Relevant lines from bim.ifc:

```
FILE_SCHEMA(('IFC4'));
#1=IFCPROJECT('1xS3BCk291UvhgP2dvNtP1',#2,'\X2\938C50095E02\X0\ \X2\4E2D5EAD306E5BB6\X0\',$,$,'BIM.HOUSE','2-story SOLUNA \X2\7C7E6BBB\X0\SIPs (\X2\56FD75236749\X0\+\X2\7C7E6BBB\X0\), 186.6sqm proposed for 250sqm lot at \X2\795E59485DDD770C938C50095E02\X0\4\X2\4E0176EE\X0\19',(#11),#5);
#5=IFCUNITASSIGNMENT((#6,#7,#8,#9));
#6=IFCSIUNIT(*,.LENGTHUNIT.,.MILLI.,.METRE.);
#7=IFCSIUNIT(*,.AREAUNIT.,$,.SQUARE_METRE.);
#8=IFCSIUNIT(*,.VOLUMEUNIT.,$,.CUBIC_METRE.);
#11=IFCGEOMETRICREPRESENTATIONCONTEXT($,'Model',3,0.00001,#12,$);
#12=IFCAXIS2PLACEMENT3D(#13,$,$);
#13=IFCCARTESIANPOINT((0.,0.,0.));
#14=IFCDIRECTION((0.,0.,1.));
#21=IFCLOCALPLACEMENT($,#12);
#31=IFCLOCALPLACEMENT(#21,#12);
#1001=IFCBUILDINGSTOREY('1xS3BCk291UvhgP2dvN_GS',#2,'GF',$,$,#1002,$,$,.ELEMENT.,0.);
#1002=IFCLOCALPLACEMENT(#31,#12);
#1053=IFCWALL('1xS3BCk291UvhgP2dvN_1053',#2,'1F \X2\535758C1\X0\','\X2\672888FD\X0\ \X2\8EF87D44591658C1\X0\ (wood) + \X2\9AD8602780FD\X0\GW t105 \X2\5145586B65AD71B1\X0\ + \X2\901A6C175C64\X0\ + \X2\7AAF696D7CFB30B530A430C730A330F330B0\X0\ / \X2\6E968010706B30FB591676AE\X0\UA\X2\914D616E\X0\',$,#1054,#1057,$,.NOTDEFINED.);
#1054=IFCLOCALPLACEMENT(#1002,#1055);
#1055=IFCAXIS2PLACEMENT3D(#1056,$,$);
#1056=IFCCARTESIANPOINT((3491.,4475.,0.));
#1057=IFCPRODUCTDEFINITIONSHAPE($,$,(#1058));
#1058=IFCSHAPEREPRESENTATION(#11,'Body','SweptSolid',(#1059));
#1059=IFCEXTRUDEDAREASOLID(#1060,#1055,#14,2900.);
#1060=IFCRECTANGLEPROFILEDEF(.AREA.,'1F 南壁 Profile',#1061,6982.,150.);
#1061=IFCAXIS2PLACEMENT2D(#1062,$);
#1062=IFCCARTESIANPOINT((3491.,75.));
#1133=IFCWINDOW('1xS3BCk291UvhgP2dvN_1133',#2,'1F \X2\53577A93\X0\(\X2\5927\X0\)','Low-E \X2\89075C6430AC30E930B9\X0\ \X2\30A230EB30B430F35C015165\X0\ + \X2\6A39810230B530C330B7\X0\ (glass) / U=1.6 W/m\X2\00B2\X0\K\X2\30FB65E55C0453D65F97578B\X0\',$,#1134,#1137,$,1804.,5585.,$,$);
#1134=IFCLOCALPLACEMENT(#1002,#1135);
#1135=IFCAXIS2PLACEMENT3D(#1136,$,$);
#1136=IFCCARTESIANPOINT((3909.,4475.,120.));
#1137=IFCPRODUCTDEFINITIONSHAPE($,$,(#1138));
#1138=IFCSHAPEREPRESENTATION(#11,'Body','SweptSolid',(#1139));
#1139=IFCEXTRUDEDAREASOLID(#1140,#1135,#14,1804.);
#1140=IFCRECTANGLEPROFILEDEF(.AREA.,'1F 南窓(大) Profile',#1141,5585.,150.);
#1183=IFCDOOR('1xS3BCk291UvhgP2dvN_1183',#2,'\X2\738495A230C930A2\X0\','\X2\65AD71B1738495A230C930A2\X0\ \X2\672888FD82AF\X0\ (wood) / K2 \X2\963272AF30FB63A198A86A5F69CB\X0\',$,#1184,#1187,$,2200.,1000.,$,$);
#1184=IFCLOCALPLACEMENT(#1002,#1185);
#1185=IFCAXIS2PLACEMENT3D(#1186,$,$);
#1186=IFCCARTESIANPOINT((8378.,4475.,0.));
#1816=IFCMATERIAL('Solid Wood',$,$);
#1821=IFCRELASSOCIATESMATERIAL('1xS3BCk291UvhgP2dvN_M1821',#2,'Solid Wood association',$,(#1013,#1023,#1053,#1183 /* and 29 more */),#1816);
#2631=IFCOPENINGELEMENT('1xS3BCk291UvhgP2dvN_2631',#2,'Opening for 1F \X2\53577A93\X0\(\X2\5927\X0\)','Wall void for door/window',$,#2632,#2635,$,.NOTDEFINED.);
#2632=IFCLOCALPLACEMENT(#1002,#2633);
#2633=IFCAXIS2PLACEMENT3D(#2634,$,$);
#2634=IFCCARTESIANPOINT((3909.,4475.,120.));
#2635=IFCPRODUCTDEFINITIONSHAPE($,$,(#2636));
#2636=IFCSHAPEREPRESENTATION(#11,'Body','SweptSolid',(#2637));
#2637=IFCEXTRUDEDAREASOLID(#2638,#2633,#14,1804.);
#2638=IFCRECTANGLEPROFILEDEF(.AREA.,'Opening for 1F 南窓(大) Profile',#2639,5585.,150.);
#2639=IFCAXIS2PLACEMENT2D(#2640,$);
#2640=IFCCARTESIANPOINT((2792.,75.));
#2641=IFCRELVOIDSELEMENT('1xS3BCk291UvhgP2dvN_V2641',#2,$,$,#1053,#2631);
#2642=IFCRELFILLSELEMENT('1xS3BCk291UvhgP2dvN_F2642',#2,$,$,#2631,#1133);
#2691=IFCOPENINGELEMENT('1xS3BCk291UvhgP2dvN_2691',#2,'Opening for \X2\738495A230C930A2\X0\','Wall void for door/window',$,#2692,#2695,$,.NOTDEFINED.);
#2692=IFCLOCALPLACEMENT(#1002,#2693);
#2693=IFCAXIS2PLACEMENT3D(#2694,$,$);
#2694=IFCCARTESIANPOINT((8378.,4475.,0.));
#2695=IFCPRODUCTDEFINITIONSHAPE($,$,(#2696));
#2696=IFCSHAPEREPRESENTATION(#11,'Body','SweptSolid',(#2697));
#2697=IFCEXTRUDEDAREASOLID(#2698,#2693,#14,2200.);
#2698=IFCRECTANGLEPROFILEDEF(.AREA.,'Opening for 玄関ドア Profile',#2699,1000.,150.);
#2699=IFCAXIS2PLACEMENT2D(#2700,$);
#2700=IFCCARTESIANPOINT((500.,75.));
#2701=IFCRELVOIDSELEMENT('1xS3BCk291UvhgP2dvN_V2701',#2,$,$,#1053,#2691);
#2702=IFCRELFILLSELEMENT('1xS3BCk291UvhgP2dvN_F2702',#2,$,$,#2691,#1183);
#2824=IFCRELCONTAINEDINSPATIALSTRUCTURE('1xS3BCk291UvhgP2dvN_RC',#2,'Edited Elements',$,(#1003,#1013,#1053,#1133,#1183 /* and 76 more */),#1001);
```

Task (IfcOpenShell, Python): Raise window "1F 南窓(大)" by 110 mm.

```python
import numpy as np
import ifcopenshell
import ifcopenshell.api.geometry
import ifcopenshell.util.placement
import ifcopenshell.util.unit

model = ifcopenshell.open("bim.ifc")
unit_scale = ifcopenshell.util.unit.calculate_unit_scale(model)

window = model.by_guid("1xS3BCk291UvhgP2dvN_1133")
opening = window.FillsVoids[0].RelatingOpeningElement
dz = 0.11 / unit_scale

shift = np.array([0.0, 0.0, dz])
# The window is not placed relative to its opening, so move both.
for product in (opening, window):
    matrix = ifcopenshell.util.placement.get_local_placement(product.ObjectPlacement)
    matrix[:3, 3] += shift
    ifcopenshell.api.geometry.edit_object_placement(model, product=product, matrix=matrix, is_si=False)

print(f"moved by {dz * unit_scale:+.3f} m")

model.write("bim_v2.ifc")
```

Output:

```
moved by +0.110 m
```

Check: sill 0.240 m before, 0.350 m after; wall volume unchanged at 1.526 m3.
